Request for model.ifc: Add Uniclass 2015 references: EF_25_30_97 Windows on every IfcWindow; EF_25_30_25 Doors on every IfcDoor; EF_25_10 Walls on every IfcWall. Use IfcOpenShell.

First a look at what the model holds.

```python
import ifcopenshell

model = ifcopenshell.open("model.ifc")
print(model.schema)
print("classifications:", [c.Name for c in model.by_type("IfcClassification")])
for ifc_class in ("IfcDoor", "IfcRoof", "IfcStair", "IfcWall", "IfcWindow"):
    print(ifc_class, len(model.by_type(ifc_class)))
```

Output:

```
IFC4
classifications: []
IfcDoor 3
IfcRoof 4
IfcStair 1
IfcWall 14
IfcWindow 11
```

```python
import ifcopenshell
import ifcopenshell.api.classification

model = ifcopenshell.open("model.ifc")

system = ifcopenshell.api.classification.add_classification(model, classification="Uniclass 2015")

codes = {
    "IfcWindow": ("EF_25_30_97", "Windows"),
    "IfcDoor": ("EF_25_30_25", "Doors"),
    "IfcWall": ("EF_25_10", "Walls"),
}
for ifc_class, (code, name) in codes.items():
    products = model.by_type(ifc_class)
    ifcopenshell.api.classification.add_reference(
        model, products=products, classification=system, identification=code, name=name
    )
    print(code, len(products))

model.write("model_rev.ifc")
```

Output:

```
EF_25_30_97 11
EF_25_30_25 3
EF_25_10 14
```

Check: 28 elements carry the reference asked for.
